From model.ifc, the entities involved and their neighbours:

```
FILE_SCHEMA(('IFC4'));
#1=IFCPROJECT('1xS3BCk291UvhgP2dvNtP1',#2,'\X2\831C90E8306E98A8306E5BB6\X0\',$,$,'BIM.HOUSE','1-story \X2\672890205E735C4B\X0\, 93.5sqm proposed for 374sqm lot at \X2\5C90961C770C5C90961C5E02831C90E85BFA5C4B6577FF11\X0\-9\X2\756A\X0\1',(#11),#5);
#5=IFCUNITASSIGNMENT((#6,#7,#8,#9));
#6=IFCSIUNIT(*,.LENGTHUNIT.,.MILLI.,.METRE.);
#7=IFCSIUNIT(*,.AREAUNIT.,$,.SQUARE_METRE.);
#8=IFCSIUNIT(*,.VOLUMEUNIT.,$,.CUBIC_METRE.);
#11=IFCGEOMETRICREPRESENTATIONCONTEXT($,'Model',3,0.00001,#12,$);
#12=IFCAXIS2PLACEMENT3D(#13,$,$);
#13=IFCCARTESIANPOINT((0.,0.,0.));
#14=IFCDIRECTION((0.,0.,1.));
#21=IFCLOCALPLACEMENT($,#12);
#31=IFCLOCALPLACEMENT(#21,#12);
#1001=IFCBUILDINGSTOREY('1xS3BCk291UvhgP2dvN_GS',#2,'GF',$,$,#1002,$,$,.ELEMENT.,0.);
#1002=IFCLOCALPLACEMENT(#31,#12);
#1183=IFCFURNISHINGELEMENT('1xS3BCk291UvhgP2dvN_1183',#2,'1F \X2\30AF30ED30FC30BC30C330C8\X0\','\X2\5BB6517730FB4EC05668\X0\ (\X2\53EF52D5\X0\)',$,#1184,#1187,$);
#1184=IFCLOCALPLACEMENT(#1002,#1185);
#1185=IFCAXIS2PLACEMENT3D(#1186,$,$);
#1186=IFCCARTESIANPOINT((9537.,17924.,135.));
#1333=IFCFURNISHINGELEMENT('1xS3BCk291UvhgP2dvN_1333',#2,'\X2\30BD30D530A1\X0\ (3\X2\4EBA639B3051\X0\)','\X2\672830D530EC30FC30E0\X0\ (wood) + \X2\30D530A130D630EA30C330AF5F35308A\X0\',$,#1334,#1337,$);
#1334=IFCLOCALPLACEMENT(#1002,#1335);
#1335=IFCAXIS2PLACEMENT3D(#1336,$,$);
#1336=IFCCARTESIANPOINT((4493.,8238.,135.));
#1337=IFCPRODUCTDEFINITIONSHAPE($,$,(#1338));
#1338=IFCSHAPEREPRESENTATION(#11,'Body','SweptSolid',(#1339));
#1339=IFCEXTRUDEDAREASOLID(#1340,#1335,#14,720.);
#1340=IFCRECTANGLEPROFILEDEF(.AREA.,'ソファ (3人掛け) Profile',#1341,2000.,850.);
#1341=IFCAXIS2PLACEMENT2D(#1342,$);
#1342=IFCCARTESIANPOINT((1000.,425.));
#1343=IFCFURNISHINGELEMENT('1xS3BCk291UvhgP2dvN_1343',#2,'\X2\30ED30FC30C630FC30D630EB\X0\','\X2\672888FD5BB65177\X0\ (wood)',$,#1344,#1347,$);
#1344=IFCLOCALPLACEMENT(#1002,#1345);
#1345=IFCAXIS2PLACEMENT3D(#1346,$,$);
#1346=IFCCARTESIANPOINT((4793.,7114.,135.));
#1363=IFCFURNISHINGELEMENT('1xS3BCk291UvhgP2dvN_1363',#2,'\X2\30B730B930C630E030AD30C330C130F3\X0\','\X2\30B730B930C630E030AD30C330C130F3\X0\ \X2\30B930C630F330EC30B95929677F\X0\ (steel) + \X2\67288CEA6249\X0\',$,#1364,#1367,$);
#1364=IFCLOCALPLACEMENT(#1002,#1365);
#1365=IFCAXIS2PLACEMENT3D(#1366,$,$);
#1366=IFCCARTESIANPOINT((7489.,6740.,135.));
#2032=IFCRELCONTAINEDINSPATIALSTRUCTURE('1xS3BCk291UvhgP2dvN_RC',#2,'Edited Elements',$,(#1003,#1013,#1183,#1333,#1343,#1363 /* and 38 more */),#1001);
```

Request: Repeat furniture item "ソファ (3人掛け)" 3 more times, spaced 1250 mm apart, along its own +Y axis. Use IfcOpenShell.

```python
import ifcopenshell
import ifcopenshell.api.geometry
import ifcopenshell.api.root
import ifcopenshell.util.element
import ifcopenshell.util.placement
import ifcopenshell.util.unit

model = ifcopenshell.open("model.ifc")
unit_scale = ifcopenshell.util.unit.calculate_unit_scale(model)


def reuse_history(source, copy):
    """copy_class also copies each property set's owner history, people and application; keep the originals."""
    for rel in copy.IsDefinedBy:
        if rel.is_a("IfcRelDefinesByProperties") and (history := rel.RelatingPropertyDefinition.OwnerHistory):
            rel.RelatingPropertyDefinition.OwnerHistory = source.OwnerHistory
            ifcopenshell.util.element.remove_deep2(model, history)


source = model.by_id(1333)
base = ifcopenshell.util.placement.get_local_placement(source.ObjectPlacement)
step = base[:3, 1] * 1.25 / unit_scale

for i in range(1, 4):
    copy = ifcopenshell.api.root.copy_class(model, product=source)
    copy.Representation = ifcopenshell.util.element.copy_deep(
        model, source.Representation, exclude=["IfcGeometricRepresentationContext", "IfcRepresentationMap"]
    )
    reuse_history(source, copy)
    matrix = base.copy()
    matrix[:3, 3] += i * step
    print("added at", matrix[:3, 3].round(3) + 0.0)
    ifcopenshell.api.geometry.edit_object_placement(model, product=copy, matrix=matrix, is_si=False)

model.write("model-out.ifc")
```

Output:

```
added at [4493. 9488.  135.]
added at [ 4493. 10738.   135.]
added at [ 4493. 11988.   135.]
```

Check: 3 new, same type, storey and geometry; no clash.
